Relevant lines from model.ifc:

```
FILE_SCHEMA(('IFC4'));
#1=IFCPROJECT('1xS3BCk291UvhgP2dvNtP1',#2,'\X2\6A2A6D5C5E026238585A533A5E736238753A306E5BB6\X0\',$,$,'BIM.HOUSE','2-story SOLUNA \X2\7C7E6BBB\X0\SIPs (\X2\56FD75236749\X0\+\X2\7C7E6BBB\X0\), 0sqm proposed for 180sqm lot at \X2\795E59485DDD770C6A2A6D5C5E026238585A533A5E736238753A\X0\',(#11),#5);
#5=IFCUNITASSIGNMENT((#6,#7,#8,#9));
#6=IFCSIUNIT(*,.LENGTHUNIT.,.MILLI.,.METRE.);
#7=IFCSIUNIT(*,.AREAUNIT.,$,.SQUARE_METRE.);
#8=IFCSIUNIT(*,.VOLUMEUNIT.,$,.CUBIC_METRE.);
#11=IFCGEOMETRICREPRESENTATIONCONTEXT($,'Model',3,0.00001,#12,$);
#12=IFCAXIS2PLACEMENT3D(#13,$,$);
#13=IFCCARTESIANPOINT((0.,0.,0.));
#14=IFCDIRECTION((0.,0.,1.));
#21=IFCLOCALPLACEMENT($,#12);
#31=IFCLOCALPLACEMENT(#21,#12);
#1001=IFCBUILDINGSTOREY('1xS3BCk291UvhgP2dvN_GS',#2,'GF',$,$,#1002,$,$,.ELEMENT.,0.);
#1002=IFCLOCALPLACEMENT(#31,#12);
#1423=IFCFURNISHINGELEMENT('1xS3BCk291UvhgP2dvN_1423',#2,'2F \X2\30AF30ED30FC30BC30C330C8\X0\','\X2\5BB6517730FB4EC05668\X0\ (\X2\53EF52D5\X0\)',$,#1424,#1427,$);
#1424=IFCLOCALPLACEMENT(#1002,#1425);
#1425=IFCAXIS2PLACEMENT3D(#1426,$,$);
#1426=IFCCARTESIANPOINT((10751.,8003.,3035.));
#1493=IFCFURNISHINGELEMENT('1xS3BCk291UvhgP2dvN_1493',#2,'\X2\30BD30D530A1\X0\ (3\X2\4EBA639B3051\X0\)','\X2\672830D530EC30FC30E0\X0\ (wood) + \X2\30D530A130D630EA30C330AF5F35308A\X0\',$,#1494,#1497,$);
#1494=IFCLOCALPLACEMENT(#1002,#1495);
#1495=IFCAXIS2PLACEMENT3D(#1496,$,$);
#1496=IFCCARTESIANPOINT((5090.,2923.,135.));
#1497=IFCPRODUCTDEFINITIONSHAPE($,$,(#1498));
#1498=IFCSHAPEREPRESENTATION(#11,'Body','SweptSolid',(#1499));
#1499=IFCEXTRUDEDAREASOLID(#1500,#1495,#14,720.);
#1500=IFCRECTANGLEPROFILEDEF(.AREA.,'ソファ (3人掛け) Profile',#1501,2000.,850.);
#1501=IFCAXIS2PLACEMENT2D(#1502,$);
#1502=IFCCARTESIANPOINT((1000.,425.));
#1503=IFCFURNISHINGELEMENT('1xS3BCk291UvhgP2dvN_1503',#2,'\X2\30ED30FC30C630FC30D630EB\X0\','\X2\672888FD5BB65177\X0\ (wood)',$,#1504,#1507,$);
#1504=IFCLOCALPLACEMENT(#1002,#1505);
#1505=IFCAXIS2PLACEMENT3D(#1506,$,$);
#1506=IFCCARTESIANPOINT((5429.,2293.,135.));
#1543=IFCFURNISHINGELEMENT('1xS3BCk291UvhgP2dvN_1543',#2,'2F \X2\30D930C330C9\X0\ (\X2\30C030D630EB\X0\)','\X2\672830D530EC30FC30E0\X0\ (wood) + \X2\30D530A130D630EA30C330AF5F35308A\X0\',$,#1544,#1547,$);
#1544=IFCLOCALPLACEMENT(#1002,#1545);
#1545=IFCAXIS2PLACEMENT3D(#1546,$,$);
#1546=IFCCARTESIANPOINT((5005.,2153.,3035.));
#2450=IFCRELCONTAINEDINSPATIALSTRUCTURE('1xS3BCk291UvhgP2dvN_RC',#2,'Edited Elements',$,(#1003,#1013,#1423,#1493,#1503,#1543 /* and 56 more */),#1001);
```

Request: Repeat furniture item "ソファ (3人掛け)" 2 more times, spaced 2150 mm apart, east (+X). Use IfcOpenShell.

```python
import numpy as np
import ifcopenshell
import ifcopenshell.api.geometry
import ifcopenshell.api.root
import ifcopenshell.util.element
import ifcopenshell.util.placement

model = ifcopenshell.open("model.ifc")


def reuse_history(source, copy):
    """copy_class also copies each property set's owner history, people and application; keep the originals."""
    for rel in copy.IsDefinedBy:
        if rel.is_a("IfcRelDefinesByProperties") and (history := rel.RelatingPropertyDefinition.OwnerHistory):
            rel.RelatingPropertyDefinition.OwnerHistory = source.OwnerHistory
            ifcopenshell.util.element.remove_deep2(model, history)


source = model.by_guid("1xS3BCk291UvhgP2dvN_1493")
base = ifcopenshell.util.placement.get_local_placement(source.ObjectPlacement)
step = np.array([1.0, 0.0, 0.0]) * 2150.0

for i in range(1, 3):
    copy = ifcopenshell.api.root.copy_class(model, product=source)
    copy.Representation = ifcopenshell.util.element.copy_deep(
        model, source.Representation, exclude=["IfcGeometricRepresentationContext", "IfcRepresentationMap"]
    )
    reuse_history(source, copy)
    matrix = base.copy()
    matrix[:3, 3] += i * step
    print("added at", matrix[:3, 3].round(3) + 0.0)
    ifcopenshell.api.geometry.edit_object_placement(model, product=copy, matrix=matrix, is_si=False)

model.write("model_updated.ifc")
```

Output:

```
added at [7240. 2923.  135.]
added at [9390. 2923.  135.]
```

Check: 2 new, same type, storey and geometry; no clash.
